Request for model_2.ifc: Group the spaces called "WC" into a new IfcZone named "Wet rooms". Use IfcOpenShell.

First a look at what the model holds.

```python
import ifcopenshell

model = ifcopenshell.open("model_2.ifc")
print(model.schema)
seen = {}
for space in model.by_type("IfcSpace"):
    seen[space.LongName] = seen.get(space.LongName, 0) + 1
for name, count in sorted(seen.items(), key=str):
    print(count, "x", name)
print("zones:", [z.Name for z in model.by_type("IfcZone")][:20])
```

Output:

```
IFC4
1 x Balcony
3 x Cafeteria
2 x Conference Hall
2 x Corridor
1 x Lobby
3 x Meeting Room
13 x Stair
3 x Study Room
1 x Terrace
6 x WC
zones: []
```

```python
import ifcopenshell
import ifcopenshell.api.group
import ifcopenshell.api.root

model = ifcopenshell.open("model_2.ifc")

names = {"WC"}
spaces = [s for s in model.by_type("IfcSpace") if s.LongName in names]

zone = ifcopenshell.api.root.create_entity(model, ifc_class="IfcZone", name="Wet rooms")
ifcopenshell.api.group.assign_group(model, products=spaces, group=zone)
print(len(spaces), "spaces in", zone.Name)

model.write("model_2_updated.ifc")
```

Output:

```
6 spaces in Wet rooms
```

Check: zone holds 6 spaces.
